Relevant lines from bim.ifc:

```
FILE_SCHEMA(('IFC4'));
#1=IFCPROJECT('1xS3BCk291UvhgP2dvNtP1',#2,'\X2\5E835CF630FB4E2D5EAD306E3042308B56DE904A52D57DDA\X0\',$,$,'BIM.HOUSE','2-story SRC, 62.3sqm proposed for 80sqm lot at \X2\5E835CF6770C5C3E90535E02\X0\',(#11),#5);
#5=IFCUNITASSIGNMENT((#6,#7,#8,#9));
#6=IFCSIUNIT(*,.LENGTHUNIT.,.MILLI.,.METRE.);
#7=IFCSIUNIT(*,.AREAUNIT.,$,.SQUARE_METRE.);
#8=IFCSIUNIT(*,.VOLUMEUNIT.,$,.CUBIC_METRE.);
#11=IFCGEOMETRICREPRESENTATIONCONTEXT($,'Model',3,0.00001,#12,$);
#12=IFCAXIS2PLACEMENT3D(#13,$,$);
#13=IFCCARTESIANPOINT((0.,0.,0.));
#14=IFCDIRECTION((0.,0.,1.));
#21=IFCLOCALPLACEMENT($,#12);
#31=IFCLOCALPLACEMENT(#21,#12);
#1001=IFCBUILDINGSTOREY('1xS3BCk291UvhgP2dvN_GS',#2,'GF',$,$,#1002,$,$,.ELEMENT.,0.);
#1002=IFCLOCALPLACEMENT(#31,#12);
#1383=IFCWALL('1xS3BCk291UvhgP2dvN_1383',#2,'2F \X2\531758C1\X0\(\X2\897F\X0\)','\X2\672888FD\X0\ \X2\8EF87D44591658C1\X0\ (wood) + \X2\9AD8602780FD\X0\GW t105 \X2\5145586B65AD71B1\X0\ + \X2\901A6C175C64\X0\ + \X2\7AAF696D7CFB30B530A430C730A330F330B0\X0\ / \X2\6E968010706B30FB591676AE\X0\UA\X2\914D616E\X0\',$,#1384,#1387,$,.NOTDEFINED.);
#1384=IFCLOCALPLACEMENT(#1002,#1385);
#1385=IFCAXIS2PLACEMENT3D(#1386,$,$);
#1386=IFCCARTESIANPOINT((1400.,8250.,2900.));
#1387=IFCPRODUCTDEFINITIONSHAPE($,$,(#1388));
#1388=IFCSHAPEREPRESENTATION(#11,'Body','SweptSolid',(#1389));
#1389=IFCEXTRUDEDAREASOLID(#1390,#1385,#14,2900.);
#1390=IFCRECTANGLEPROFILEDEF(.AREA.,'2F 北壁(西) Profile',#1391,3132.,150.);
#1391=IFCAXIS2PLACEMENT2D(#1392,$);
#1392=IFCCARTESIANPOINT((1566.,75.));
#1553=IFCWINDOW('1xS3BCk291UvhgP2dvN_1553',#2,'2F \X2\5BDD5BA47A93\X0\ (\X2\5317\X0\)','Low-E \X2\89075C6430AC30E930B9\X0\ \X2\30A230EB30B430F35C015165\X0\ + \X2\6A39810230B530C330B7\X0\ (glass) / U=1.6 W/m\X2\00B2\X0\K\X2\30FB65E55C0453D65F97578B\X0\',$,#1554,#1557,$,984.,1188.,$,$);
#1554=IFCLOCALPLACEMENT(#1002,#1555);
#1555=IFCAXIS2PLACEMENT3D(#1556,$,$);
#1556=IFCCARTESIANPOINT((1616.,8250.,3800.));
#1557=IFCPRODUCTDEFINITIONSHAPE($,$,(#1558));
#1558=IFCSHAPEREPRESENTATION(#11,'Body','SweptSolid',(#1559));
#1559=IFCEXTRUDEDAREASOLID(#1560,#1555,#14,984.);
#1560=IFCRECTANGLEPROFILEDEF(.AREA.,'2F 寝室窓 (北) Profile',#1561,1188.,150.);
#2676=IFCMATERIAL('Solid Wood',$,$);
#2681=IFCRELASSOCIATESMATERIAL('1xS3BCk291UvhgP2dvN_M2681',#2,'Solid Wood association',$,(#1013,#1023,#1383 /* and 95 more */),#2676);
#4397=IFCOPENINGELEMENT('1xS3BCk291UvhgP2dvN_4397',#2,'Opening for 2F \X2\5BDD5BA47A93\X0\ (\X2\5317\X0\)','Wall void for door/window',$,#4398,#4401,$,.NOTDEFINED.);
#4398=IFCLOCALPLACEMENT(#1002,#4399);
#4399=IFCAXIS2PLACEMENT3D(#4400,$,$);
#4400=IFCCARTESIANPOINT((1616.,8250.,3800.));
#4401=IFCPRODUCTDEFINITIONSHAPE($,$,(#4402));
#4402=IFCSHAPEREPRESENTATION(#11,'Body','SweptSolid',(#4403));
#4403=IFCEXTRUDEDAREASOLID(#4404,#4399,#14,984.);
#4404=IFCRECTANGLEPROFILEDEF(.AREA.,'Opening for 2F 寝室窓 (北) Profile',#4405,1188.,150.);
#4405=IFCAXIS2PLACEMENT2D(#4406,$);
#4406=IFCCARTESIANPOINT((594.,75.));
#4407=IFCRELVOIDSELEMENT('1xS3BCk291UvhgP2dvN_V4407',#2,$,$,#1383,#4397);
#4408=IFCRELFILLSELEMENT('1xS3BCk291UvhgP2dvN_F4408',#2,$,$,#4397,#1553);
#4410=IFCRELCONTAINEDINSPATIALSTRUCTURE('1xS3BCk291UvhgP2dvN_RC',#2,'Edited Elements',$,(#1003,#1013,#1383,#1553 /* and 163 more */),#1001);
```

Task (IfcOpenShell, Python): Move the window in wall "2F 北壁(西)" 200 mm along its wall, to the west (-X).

```python
import ifcopenshell
import ifcopenshell.api.geometry
import ifcopenshell.util.placement

model = ifcopenshell.open("bim.ifc")

window = model.by_guid("1xS3BCk291UvhgP2dvN_1553")
opening = window.FillsVoids[0].RelatingOpeningElement
wall = opening.VoidsElements[0].RelatingBuildingElement

wall_matrix = ifcopenshell.util.placement.get_local_placement(wall.ObjectPlacement)
shift = wall_matrix[:3, 0] * -200.0
before = ifcopenshell.util.placement.get_local_placement(window.ObjectPlacement)[:3, 3].copy()

# The window is not placed relative to its opening, so move both.
for product in (opening, window):
    matrix = ifcopenshell.util.placement.get_local_placement(product.ObjectPlacement)
    matrix[:3, 3] += shift
    ifcopenshell.api.geometry.edit_object_placement(model, product=product, matrix=matrix, is_si=False)

after = ifcopenshell.util.placement.get_local_placement(window.ObjectPlacement)[:3, 3]
print("window moved by", (after - before).round(3) + 0.0)

model.write("bim_rev.ifc")
```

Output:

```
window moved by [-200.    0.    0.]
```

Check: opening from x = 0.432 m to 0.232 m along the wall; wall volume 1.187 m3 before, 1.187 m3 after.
